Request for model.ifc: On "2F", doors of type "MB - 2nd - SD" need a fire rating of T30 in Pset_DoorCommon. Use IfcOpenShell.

First a look at what the model holds.

```python
import ifcopenshell
import ifcopenshell.util.element

model = ifcopenshell.open("model.ifc")
print(model.schema)
storey = next(s for s in model.by_type("IfcBuildingStorey") if s.Name == "2F")
doors = [e for e in ifcopenshell.util.element.get_decomposition(storey) if e.is_a("IfcDoor")]
seen = {}
for e in doors:
    element_type = ifcopenshell.util.element.get_type(e)
    key = (element_type.Name if element_type != e and element_type else None, ifcopenshell.util.element.get_pset(e, "Pset_DoorCommon", "FireRating"))
    seen[key] = seen.get(key, 0) + 1
for (name, value), count in sorted(seen.items(), key=str):
    print(count, "x", name, "|", value)
```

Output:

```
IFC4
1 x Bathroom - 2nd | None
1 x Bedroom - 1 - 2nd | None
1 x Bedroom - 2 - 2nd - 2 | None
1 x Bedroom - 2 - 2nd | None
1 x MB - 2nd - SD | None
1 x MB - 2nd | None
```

```python
import ifcopenshell
import ifcopenshell.api.pset
import ifcopenshell.util.element

model = ifcopenshell.open("model.ifc")

storey = next(s for s in model.by_type("IfcBuildingStorey") if s.Name == "2F")
doors = [e for e in ifcopenshell.util.element.get_decomposition(storey) if e.is_a("IfcDoor")]

count = 0
for e in doors:
    element_type = ifcopenshell.util.element.get_type(e)
    if element_type in (None, e) or element_type.Name != "MB - 2nd - SD":
        continue
    # add_pset returns the element's existing set when there is one.
    pset = ifcopenshell.api.pset.add_pset(model, product=e, name="Pset_DoorCommon")
    ifcopenshell.api.pset.edit_pset(model, pset=pset, properties={"FireRating": "T30"})
    count += 1

print(count, "doors updated")

model.write("model_edited.ifc")
```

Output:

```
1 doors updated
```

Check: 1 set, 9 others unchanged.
